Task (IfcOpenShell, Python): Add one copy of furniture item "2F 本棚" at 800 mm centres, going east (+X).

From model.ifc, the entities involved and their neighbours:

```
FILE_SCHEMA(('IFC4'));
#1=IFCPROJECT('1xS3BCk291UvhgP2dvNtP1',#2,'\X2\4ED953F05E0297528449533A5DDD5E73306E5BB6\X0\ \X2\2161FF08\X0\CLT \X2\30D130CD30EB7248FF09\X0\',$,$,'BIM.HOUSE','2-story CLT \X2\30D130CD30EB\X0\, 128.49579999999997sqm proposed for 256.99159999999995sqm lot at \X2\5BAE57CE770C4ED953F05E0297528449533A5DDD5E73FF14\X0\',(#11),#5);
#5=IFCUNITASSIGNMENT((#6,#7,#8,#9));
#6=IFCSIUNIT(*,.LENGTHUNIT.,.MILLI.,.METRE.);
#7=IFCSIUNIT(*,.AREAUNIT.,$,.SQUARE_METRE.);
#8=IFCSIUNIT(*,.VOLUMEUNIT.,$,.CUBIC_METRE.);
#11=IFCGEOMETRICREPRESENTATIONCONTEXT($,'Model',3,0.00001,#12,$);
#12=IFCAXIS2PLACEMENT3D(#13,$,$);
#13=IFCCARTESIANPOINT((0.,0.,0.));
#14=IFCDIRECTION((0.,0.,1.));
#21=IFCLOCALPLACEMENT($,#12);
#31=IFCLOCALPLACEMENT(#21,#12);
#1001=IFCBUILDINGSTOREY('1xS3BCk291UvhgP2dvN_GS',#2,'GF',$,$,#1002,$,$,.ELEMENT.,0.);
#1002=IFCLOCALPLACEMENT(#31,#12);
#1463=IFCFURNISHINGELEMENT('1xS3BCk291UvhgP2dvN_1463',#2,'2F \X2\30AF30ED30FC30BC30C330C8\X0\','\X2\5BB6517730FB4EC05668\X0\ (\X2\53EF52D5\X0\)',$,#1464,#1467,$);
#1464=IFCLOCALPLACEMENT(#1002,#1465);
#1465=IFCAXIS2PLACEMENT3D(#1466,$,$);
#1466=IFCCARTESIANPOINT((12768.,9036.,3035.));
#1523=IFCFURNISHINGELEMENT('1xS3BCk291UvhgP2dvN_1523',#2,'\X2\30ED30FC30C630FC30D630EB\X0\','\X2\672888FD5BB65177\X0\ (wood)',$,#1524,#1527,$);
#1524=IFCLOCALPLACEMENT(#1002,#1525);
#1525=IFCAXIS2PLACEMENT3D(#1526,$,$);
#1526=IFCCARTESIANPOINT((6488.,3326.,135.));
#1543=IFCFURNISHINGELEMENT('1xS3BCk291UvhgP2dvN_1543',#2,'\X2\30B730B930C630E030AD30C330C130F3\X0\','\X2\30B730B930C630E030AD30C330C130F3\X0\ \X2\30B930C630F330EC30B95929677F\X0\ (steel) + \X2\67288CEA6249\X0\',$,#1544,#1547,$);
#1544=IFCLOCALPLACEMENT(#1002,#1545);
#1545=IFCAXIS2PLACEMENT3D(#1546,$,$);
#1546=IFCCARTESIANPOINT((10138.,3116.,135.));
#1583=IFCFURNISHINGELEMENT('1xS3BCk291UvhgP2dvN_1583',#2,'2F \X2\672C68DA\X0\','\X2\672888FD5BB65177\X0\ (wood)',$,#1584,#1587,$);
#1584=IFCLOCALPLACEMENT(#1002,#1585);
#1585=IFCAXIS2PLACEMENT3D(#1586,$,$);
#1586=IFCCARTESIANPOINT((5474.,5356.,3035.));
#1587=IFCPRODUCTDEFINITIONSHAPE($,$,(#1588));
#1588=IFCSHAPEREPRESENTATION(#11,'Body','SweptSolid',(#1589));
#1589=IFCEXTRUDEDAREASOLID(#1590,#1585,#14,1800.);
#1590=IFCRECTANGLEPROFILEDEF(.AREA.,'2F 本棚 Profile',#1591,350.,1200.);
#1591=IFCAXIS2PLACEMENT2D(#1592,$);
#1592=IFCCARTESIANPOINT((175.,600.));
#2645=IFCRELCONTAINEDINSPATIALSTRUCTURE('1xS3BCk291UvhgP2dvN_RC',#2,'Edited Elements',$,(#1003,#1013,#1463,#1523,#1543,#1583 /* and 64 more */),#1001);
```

```python
import numpy as np
import ifcopenshell
import ifcopenshell.api.geometry
import ifcopenshell.api.root
import ifcopenshell.util.element
import ifcopenshell.util.placement
import ifcopenshell.util.unit

model = ifcopenshell.open("model.ifc")
unit_scale = ifcopenshell.util.unit.calculate_unit_scale(model)


def reuse_history(source, copy):
    """copy_class also copies each property set's owner history, people and application; keep the originals."""
    for rel in copy.IsDefinedBy:
        if rel.is_a("IfcRelDefinesByProperties") and (history := rel.RelatingPropertyDefinition.OwnerHistory):
            rel.RelatingPropertyDefinition.OwnerHistory = source.OwnerHistory
            ifcopenshell.util.element.remove_deep2(model, history)


source = model.by_guid("1xS3BCk291UvhgP2dvN_1583")
base = ifcopenshell.util.placement.get_local_placement(source.ObjectPlacement)
step = np.array([1.0, 0.0, 0.0]) * 0.8 / unit_scale

for i in range(1, 2):
    copy = ifcopenshell.api.root.copy_class(model, product=source)
    copy.Representation = ifcopenshell.util.element.copy_deep(
        model, source.Representation, exclude=["IfcGeometricRepresentationContext", "IfcRepresentationMap"]
    )
    reuse_history(source, copy)
    matrix = base.copy()
    matrix[:3, 3] += i * step
    print("added at", matrix[:3, 3].round(3) + 0.0)
    ifcopenshell.api.geometry.edit_object_placement(model, product=copy, matrix=matrix, is_si=False)

model.write("model_v2.ifc")
```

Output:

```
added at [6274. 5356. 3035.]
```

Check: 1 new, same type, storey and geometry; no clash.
